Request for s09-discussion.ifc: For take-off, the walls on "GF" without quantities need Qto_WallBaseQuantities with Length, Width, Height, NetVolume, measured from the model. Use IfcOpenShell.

First a look at what the model holds.

```python
import ifcopenshell
import ifcopenshell.util.element
import ifcopenshell.util.unit

model = ifcopenshell.open("s09-discussion.ifc")
print(model.schema)
for unit_type in ("LENGTHUNIT", "AREAUNIT", "VOLUMEUNIT"):
    print(unit_type, ifcopenshell.util.unit.calculate_unit_scale(model, unit_type))
storey = next(s for s in model.by_type("IfcBuildingStorey") if s.Name == "GF")
walls = [e for e in ifcopenshell.util.element.get_decomposition(storey) if e.is_a("IfcWall")]
for e in sorted(walls, key=lambda e: e.id()):
    print(e.id(), e.is_a(), e.Name, list(ifcopenshell.util.element.get_psets(e, qtos_only=True)), sep=" | ")
```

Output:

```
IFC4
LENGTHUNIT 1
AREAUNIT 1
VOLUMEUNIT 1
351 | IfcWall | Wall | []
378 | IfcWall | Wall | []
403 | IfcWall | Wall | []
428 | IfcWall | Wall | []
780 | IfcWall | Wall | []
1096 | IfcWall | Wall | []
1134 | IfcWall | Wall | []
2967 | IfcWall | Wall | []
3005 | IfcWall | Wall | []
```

```python
import ifcopenshell
import ifcopenshell.api.pset
import ifcopenshell.geom
import ifcopenshell.util.element
import ifcopenshell.util.shape
import ifcopenshell.util.unit

model = ifcopenshell.open("s09-discussion.ifc")
unit_scale = ifcopenshell.util.unit.calculate_unit_scale(model)
volume_scale = ifcopenshell.util.unit.calculate_unit_scale(model, "VOLUMEUNIT")
settings = ifcopenshell.geom.settings()

storey = next(s for s in model.by_type("IfcBuildingStorey") if s.Name == "GF")
walls = [e for e in ifcopenshell.util.element.get_decomposition(storey) if e.is_a("IfcWall")]

for e in sorted(walls, key=lambda e: e.id()):
    if ifcopenshell.util.element.get_psets(e, qtos_only=True, should_inherit=False):
        continue
    # Geometry comes back in metres, in the element's own axes.
    shape = ifcopenshell.geom.create_shape(settings, e)
    values = {
        "Length": ifcopenshell.util.shape.get_x(shape.geometry) / unit_scale,
        "Width": ifcopenshell.util.shape.get_y(shape.geometry) / unit_scale,
        "Height": ifcopenshell.util.shape.get_z(shape.geometry) / unit_scale,
        "NetVolume": ifcopenshell.util.shape.get_volume(shape.geometry) / volume_scale,
    }
    qto = ifcopenshell.api.pset.add_qto(model, product=e, name="Qto_WallBaseQuantities")
    ifcopenshell.api.pset.edit_qto(model, qto=qto, properties=values)
    print(e.id(), {k: round(v, 3) for k, v in values.items()})

model.write("s09-discussion_updated.ifc")
```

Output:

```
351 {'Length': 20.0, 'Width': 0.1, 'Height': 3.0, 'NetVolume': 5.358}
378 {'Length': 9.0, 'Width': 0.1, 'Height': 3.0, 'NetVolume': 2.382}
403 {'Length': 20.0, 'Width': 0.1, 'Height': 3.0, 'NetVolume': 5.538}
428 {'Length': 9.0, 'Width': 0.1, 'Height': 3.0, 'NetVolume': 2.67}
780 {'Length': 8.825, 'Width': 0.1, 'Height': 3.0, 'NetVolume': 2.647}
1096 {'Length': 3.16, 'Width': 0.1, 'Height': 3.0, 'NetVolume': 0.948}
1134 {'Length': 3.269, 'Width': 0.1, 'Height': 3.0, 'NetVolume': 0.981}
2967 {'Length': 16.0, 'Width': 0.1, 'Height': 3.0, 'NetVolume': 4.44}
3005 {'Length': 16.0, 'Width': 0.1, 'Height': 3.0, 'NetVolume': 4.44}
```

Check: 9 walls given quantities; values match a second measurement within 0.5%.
